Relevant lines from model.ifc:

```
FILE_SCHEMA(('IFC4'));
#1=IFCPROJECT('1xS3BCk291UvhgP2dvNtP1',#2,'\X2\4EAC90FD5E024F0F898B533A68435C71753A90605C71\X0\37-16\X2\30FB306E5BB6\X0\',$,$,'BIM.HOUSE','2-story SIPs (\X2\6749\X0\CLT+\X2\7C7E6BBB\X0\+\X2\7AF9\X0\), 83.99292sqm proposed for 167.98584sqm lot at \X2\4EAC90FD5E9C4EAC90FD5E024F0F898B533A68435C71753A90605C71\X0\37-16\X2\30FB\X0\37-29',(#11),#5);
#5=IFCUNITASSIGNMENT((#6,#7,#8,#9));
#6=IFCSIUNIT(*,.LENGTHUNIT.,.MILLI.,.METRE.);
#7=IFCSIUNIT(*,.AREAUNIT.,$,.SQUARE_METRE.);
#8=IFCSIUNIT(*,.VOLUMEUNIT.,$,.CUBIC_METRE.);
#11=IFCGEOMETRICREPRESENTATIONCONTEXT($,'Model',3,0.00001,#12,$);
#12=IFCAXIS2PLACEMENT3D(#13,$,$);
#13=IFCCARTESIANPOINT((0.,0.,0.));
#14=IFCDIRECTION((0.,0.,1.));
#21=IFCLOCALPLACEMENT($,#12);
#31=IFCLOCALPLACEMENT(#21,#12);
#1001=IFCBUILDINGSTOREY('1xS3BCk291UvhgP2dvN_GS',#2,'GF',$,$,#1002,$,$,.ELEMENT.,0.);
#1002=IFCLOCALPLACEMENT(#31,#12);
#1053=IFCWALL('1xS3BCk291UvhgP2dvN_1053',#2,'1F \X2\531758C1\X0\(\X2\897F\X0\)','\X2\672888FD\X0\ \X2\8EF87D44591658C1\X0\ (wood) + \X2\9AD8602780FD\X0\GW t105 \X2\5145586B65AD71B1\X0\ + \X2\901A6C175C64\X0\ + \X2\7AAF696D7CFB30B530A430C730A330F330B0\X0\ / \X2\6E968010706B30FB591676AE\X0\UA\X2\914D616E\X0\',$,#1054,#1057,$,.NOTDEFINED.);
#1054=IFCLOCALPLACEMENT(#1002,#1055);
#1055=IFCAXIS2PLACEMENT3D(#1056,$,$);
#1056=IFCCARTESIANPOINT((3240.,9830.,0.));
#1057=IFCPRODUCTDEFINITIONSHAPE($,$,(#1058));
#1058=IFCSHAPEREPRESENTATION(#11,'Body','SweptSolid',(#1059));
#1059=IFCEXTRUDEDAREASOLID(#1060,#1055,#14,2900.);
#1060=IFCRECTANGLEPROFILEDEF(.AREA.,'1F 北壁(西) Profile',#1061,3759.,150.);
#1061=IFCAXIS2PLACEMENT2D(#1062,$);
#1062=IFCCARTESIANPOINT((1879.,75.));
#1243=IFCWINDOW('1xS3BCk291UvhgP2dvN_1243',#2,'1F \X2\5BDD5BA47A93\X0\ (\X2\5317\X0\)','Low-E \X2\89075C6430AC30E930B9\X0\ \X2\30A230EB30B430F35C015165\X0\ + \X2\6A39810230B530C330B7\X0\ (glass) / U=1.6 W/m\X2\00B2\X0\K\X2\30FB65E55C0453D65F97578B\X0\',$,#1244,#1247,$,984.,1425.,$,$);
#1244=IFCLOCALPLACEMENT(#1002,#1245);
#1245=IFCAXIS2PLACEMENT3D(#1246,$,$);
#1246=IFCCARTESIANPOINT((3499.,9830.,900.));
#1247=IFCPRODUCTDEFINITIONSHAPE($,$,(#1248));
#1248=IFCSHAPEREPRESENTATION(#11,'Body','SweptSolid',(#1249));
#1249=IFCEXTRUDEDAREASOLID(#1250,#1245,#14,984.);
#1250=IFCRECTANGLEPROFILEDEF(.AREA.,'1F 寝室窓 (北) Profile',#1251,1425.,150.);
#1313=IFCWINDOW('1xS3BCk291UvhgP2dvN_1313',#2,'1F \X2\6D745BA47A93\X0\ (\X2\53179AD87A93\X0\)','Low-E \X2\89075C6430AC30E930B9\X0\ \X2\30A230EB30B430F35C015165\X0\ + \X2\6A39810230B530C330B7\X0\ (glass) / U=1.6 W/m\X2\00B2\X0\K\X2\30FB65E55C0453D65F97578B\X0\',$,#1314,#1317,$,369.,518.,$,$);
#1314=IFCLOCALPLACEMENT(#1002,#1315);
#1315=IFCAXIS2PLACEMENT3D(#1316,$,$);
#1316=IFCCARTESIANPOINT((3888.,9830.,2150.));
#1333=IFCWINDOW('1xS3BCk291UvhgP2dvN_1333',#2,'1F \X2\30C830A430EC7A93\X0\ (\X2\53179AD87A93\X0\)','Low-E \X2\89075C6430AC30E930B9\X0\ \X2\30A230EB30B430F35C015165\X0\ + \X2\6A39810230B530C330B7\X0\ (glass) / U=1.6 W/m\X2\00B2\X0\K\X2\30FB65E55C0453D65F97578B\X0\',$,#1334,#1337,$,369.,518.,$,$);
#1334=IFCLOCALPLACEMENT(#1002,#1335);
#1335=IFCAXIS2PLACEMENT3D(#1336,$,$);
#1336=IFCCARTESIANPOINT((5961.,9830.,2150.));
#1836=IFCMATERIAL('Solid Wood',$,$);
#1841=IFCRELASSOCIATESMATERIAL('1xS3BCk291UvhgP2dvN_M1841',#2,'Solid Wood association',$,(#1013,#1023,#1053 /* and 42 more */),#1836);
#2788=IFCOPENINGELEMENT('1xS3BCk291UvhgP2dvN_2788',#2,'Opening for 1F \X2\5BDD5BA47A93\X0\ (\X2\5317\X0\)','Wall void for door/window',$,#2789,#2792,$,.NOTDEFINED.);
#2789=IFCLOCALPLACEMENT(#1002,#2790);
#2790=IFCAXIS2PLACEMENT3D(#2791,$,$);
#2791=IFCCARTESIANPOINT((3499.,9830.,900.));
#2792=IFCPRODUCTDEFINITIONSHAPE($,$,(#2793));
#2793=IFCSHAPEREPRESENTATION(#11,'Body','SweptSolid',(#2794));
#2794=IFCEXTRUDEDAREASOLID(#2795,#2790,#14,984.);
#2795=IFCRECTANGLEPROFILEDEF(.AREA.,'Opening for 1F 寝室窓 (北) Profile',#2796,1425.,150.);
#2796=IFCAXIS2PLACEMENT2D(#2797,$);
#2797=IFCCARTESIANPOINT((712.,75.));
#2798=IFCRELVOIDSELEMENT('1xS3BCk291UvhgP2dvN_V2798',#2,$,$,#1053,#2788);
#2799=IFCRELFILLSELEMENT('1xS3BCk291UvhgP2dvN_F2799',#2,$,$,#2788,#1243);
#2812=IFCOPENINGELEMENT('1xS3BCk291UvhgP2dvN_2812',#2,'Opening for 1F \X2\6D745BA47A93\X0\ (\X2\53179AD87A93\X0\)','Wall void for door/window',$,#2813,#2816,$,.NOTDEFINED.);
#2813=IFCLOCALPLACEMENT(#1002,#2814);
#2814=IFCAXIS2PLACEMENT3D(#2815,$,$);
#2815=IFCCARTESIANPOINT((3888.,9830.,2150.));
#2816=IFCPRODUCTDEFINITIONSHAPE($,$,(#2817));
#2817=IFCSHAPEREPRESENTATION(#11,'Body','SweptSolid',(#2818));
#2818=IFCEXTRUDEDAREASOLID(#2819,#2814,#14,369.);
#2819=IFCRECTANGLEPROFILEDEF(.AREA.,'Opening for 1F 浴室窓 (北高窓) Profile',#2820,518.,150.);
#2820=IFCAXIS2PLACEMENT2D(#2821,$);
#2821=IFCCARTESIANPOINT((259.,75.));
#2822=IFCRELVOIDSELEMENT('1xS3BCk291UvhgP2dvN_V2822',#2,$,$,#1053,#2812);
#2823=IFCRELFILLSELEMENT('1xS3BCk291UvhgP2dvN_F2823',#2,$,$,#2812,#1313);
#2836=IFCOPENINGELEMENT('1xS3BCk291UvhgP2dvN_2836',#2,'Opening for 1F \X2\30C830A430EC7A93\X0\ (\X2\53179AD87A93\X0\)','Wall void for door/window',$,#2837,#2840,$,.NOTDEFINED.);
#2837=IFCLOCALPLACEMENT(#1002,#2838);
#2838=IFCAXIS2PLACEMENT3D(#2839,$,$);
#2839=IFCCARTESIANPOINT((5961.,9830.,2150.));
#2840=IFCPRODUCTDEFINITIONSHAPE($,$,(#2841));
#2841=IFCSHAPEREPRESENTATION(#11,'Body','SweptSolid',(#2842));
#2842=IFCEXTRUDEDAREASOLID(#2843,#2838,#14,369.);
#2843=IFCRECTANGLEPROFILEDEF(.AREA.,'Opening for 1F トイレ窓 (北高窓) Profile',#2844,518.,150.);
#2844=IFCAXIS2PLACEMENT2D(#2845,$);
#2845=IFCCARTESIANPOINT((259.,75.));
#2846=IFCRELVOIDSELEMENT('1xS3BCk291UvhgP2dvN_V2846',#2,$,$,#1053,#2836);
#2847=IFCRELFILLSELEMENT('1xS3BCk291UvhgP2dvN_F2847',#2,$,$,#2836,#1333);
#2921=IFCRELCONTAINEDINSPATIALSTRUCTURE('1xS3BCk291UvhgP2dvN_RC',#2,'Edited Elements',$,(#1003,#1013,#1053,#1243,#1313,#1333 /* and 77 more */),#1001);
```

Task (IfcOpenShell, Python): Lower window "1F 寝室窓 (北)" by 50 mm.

```python
import numpy as np
import ifcopenshell
import ifcopenshell.api.geometry
import ifcopenshell.util.placement
import ifcopenshell.util.unit

model = ifcopenshell.open("model.ifc")
unit_scale = ifcopenshell.util.unit.calculate_unit_scale(model)

window = model.by_guid("1xS3BCk291UvhgP2dvN_1243")
opening = window.FillsVoids[0].RelatingOpeningElement
dz = -0.05 / unit_scale

shift = np.array([0.0, 0.0, dz])
# The window is not placed relative to its opening, so move both.
for product in (opening, window):
    matrix = ifcopenshell.util.placement.get_local_placement(product.ObjectPlacement)
    matrix[:3, 3] += shift
    ifcopenshell.api.geometry.edit_object_placement(model, product=product, matrix=matrix, is_si=False)

print(f"moved by {dz * unit_scale:+.3f} m")

model.write("model_edited.ifc")
```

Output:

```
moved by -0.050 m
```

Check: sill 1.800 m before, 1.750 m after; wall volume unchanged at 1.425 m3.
